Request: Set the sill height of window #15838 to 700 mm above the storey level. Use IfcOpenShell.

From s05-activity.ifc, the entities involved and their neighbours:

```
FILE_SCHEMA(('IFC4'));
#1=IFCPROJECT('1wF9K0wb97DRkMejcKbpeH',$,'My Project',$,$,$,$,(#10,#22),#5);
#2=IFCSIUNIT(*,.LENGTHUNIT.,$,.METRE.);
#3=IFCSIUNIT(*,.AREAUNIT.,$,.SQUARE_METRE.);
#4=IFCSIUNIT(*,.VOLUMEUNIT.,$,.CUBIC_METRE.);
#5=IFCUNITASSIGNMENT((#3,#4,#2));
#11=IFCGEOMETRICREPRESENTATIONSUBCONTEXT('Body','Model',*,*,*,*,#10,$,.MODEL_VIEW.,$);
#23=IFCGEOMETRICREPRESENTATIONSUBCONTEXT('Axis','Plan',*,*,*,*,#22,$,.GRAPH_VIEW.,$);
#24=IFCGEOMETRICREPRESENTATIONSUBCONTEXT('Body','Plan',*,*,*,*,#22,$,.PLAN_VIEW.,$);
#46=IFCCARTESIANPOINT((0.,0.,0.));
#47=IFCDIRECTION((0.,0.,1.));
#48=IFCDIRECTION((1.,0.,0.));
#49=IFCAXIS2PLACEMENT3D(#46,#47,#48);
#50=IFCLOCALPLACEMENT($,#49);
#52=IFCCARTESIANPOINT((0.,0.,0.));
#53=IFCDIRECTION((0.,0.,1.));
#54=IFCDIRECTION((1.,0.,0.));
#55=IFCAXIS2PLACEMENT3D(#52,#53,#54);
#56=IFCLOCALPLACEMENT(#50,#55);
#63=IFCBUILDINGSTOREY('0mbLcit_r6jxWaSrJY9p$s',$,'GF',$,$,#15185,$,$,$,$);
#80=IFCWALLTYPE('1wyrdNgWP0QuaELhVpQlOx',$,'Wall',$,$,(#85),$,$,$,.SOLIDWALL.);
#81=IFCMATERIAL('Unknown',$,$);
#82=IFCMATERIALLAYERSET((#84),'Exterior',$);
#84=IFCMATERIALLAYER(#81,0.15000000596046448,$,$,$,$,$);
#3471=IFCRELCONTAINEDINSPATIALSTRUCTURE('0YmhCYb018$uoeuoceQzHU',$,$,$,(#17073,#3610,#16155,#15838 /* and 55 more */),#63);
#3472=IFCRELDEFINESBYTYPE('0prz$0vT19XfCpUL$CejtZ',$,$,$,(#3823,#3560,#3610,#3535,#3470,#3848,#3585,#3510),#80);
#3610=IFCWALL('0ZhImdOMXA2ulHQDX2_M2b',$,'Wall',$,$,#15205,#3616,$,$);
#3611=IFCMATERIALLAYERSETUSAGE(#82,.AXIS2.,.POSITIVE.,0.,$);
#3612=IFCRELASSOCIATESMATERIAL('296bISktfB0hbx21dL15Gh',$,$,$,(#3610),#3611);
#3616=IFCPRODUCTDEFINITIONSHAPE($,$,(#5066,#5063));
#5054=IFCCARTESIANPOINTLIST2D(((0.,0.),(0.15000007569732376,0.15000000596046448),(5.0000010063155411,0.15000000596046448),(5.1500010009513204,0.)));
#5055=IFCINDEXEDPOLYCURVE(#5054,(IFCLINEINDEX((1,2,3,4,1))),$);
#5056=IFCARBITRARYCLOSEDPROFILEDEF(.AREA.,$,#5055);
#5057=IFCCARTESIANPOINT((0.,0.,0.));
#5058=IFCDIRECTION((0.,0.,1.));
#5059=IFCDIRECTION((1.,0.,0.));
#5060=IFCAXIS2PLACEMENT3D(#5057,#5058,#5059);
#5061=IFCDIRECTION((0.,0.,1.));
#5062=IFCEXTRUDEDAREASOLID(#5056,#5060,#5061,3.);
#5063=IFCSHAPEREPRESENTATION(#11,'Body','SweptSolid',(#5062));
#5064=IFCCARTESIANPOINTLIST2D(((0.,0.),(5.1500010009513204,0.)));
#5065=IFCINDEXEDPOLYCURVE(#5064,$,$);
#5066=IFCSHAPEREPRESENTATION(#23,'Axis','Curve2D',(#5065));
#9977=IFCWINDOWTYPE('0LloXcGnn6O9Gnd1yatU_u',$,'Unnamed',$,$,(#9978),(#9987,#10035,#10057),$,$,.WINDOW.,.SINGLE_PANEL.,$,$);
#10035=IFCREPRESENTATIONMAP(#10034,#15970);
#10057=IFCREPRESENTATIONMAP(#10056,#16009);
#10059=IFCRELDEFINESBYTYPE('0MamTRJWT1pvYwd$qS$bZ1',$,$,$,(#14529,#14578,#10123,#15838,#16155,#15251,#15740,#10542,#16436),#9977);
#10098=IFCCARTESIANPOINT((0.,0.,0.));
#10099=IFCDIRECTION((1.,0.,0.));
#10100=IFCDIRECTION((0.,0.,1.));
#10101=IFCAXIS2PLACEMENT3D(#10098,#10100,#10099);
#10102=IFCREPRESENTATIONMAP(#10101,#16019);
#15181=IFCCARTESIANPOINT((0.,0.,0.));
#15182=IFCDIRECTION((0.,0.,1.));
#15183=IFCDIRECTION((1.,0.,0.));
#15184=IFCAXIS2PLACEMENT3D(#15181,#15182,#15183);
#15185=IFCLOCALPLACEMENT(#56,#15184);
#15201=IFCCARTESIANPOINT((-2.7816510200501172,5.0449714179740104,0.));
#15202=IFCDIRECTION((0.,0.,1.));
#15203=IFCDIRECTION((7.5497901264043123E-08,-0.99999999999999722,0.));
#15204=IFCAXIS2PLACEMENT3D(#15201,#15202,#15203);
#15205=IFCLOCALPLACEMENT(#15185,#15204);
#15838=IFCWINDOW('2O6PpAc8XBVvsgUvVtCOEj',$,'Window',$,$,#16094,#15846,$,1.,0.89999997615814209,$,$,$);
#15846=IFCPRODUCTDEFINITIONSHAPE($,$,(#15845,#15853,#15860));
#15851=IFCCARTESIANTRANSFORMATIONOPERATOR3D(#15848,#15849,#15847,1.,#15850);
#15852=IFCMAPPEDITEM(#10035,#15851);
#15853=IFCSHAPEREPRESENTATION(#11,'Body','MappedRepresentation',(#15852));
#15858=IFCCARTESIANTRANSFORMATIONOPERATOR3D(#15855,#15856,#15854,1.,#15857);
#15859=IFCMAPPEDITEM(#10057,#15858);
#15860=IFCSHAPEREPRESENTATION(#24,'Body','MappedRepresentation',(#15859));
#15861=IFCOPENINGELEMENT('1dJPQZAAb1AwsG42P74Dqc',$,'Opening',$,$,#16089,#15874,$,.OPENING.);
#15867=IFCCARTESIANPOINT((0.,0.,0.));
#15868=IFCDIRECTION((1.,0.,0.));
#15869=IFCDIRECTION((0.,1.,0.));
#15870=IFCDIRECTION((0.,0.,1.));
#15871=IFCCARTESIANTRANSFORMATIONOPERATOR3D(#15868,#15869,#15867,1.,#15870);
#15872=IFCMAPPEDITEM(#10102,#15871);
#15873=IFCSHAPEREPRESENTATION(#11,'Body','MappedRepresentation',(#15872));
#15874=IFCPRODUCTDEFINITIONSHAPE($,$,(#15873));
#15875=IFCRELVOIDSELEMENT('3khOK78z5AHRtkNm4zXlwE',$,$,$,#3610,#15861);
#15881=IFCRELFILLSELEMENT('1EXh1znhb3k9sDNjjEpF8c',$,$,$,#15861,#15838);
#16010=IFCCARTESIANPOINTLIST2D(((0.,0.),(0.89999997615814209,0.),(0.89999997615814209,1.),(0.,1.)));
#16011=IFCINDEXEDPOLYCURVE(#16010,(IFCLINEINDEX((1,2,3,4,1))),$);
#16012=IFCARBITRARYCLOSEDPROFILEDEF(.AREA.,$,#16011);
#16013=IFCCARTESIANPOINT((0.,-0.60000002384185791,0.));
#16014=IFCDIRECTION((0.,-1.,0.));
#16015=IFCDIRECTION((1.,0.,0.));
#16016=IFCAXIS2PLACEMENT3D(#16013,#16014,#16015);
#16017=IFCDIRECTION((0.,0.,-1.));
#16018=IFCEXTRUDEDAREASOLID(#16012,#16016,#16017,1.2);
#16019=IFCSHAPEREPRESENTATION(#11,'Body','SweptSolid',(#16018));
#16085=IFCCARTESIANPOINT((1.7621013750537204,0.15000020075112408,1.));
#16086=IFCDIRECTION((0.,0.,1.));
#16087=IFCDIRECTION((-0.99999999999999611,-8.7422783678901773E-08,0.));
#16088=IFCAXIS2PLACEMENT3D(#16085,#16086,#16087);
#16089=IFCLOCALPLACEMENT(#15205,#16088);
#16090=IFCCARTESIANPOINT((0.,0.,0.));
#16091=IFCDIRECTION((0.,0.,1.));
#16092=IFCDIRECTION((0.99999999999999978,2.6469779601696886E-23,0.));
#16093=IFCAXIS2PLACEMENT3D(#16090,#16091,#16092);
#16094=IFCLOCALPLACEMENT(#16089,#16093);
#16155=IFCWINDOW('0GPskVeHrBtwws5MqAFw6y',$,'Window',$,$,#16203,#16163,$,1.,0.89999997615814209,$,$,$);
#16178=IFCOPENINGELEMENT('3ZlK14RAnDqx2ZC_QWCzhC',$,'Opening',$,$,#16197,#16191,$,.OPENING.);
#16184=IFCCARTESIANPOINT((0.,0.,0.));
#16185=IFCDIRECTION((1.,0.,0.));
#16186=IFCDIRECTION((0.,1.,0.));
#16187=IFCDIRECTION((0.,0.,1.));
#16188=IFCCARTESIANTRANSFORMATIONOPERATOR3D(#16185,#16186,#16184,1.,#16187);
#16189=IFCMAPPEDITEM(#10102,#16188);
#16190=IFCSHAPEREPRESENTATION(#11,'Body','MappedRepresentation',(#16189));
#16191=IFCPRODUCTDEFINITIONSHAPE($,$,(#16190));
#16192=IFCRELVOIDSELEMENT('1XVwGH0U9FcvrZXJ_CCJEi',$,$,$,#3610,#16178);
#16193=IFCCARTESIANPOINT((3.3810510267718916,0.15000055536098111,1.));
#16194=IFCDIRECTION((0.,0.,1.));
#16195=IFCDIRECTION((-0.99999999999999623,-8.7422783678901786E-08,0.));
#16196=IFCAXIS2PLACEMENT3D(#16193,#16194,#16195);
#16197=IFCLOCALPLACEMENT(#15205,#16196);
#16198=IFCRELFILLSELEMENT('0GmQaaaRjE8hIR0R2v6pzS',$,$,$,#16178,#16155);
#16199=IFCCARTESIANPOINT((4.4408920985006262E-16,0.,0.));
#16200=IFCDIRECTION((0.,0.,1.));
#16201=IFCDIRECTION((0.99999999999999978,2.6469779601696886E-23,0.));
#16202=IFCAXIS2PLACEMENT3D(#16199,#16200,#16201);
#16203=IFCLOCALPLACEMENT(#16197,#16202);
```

```python
import numpy as np
import ifcopenshell
import ifcopenshell.api.geometry
import ifcopenshell.geom
import ifcopenshell.util.element
import ifcopenshell.util.placement
import ifcopenshell.util.shape
import ifcopenshell.util.unit

model = ifcopenshell.open("s05-activity.ifc")
unit_scale = ifcopenshell.util.unit.calculate_unit_scale(model)

window = model.by_id(15838)
opening = window.FillsVoids[0].RelatingOpeningElement
storey = ifcopenshell.util.element.get_container(window, ifc_class="IfcBuildingStorey")
level = ifcopenshell.util.placement.get_local_placement(storey.ObjectPlacement)[2, 3]

# The opening's origin need not be at the sill, so measure its lowest point.
shape = ifcopenshell.geom.create_shape(ifcopenshell.geom.settings(), opening)
bottom = ifcopenshell.util.shape.get_shape_bottom_elevation(shape, shape.geometry) / unit_scale
dz = level + 0.7 - bottom

shift = np.array([0.0, 0.0, dz])
# The window is placed relative to its opening, so it follows when the opening moves.
matrix = ifcopenshell.util.placement.get_local_placement(opening.ObjectPlacement)
matrix[:3, 3] += shift
ifcopenshell.api.geometry.edit_object_placement(
    model, product=opening, matrix=matrix, is_si=False, should_transform_children=True
)

print(f"moved by {dz * unit_scale:+.3f} m")

model.write("s05-activity_edited.ifc")
```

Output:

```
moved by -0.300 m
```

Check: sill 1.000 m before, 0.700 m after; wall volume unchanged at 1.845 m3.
